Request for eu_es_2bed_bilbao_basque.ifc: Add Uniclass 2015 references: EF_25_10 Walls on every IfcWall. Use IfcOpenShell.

First a look at what the model holds.

```python
import ifcopenshell

model = ifcopenshell.open("eu_es_2bed_bilbao_basque.ifc")
print(model.schema)
print("classifications:", [c.Name for c in model.by_type("IfcClassification")])
for ifc_class in ("IfcDoor", "IfcRoof", "IfcStair", "IfcWall", "IfcWindow"):
    print(ifc_class, len(model.by_type(ifc_class)))
```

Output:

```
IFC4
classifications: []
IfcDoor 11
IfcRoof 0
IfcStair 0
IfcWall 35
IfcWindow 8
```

```python
import ifcopenshell
import ifcopenshell.api.classification

model = ifcopenshell.open("eu_es_2bed_bilbao_basque.ifc")

system = ifcopenshell.api.classification.add_classification(model, classification="Uniclass 2015")

codes = {
    "IfcWall": ("EF_25_10", "Walls"),
}
for ifc_class, (code, name) in codes.items():
    products = model.by_type(ifc_class)
    ifcopenshell.api.classification.add_reference(
        model, products=products, classification=system, identification=code, name=name
    )
    print(code, len(products))

model.write("eu_es_2bed_bilbao_basque-out.ifc")
```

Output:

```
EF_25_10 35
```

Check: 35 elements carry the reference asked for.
